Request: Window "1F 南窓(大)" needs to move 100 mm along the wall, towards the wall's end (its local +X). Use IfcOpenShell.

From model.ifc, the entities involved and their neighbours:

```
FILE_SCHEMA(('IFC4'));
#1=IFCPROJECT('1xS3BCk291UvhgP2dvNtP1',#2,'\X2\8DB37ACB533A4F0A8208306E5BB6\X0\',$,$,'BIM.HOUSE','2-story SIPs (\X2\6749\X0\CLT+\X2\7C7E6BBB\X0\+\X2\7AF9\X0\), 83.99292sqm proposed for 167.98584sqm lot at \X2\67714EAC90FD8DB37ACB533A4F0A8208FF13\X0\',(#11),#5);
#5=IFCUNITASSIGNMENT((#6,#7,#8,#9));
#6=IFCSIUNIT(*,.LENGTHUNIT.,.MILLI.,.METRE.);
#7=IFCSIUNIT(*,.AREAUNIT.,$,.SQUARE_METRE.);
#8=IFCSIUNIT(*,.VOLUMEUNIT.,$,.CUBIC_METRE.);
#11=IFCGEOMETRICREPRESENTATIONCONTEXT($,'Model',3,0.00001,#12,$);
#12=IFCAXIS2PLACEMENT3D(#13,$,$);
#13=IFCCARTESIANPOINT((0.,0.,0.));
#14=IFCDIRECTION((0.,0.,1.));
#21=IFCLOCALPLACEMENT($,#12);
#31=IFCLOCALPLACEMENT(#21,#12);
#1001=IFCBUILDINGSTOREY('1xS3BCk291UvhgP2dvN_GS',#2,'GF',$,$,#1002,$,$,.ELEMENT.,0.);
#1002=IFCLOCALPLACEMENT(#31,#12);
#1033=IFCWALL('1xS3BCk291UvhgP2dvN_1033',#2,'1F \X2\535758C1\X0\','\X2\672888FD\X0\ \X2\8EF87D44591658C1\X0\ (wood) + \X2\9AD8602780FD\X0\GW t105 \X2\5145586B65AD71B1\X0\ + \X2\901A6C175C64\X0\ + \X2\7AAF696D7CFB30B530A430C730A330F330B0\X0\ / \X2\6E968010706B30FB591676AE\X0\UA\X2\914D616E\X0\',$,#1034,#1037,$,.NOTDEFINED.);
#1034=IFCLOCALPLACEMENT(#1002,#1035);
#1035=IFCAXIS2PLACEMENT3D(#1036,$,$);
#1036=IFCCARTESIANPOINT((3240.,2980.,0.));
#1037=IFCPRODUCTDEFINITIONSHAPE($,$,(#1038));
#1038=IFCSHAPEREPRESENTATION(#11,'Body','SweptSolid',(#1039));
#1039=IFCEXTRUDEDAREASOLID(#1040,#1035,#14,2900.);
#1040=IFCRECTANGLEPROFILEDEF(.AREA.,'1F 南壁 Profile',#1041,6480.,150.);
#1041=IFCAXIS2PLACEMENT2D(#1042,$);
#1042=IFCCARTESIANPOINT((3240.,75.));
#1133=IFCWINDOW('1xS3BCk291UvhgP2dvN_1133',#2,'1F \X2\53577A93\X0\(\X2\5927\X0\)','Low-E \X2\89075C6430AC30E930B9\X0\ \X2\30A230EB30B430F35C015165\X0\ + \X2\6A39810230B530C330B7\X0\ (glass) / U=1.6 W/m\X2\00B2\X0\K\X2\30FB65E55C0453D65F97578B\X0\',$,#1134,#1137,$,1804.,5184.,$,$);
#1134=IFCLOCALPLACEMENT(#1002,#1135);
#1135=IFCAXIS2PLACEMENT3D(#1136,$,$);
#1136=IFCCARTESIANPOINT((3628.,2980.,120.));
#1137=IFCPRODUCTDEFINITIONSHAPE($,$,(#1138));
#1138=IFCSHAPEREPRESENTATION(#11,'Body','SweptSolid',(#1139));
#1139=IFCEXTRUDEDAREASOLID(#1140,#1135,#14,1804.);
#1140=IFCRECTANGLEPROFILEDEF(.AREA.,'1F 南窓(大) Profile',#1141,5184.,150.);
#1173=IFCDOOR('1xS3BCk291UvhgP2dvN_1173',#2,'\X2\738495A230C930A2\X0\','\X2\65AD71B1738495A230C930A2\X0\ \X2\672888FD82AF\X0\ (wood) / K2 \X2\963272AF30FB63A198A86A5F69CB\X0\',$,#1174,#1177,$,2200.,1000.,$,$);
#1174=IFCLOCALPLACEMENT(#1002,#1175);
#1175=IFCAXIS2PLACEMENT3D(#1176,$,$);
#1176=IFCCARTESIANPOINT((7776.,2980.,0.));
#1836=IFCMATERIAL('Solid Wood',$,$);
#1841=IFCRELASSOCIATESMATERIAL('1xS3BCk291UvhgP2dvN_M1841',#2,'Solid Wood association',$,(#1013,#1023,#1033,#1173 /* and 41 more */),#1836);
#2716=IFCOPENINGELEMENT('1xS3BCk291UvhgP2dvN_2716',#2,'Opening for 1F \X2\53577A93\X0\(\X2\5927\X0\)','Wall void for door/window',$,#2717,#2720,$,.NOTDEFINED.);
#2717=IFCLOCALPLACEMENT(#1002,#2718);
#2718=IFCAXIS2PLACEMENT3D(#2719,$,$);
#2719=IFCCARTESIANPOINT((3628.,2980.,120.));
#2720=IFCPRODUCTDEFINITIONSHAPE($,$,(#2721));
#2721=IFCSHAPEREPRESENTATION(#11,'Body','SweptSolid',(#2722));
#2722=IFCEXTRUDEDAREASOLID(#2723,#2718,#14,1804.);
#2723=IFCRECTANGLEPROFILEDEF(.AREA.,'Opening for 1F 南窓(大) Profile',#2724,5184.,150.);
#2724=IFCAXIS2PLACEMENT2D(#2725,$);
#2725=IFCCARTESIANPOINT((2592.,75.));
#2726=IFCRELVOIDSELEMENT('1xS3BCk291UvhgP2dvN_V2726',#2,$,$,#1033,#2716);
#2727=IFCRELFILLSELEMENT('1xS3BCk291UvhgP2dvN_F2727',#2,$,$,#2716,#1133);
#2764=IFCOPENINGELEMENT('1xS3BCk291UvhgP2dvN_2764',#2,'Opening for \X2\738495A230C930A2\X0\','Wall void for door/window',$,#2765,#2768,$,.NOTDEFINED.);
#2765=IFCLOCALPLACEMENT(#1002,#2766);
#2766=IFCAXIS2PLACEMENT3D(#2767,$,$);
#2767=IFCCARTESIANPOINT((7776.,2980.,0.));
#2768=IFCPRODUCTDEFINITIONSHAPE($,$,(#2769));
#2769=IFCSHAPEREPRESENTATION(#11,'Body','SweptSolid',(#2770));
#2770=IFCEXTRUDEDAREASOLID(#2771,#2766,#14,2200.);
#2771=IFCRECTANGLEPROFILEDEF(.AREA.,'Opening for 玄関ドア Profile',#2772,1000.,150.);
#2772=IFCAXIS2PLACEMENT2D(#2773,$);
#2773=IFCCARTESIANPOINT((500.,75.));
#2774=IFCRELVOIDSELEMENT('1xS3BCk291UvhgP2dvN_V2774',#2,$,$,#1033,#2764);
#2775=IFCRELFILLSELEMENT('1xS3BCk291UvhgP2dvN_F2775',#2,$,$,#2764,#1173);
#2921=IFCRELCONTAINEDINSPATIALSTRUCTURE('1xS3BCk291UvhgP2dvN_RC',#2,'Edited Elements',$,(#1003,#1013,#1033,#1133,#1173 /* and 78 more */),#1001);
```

```python
import ifcopenshell
import ifcopenshell.api.geometry
import ifcopenshell.util.placement

model = ifcopenshell.open("model.ifc")

window = model.by_guid("1xS3BCk291UvhgP2dvN_1133")
opening = window.FillsVoids[0].RelatingOpeningElement
wall = opening.VoidsElements[0].RelatingBuildingElement

wall_matrix = ifcopenshell.util.placement.get_local_placement(wall.ObjectPlacement)
shift = wall_matrix[:3, 0] * 100.0
before = ifcopenshell.util.placement.get_local_placement(window.ObjectPlacement)[:3, 3].copy()

# The window is not placed relative to its opening, so move both.
for product in (opening, window):
    matrix = ifcopenshell.util.placement.get_local_placement(product.ObjectPlacement)
    matrix[:3, 3] += shift
    ifcopenshell.api.geometry.edit_object_placement(model, product=product, matrix=matrix, is_si=False)

after = ifcopenshell.util.placement.get_local_placement(window.ObjectPlacement)[:3, 3]
print("window moved by", (after - before).round(3) + 0.0)

model.write("model_rev.ifc")
```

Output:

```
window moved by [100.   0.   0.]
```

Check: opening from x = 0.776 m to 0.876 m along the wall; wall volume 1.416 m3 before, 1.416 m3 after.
